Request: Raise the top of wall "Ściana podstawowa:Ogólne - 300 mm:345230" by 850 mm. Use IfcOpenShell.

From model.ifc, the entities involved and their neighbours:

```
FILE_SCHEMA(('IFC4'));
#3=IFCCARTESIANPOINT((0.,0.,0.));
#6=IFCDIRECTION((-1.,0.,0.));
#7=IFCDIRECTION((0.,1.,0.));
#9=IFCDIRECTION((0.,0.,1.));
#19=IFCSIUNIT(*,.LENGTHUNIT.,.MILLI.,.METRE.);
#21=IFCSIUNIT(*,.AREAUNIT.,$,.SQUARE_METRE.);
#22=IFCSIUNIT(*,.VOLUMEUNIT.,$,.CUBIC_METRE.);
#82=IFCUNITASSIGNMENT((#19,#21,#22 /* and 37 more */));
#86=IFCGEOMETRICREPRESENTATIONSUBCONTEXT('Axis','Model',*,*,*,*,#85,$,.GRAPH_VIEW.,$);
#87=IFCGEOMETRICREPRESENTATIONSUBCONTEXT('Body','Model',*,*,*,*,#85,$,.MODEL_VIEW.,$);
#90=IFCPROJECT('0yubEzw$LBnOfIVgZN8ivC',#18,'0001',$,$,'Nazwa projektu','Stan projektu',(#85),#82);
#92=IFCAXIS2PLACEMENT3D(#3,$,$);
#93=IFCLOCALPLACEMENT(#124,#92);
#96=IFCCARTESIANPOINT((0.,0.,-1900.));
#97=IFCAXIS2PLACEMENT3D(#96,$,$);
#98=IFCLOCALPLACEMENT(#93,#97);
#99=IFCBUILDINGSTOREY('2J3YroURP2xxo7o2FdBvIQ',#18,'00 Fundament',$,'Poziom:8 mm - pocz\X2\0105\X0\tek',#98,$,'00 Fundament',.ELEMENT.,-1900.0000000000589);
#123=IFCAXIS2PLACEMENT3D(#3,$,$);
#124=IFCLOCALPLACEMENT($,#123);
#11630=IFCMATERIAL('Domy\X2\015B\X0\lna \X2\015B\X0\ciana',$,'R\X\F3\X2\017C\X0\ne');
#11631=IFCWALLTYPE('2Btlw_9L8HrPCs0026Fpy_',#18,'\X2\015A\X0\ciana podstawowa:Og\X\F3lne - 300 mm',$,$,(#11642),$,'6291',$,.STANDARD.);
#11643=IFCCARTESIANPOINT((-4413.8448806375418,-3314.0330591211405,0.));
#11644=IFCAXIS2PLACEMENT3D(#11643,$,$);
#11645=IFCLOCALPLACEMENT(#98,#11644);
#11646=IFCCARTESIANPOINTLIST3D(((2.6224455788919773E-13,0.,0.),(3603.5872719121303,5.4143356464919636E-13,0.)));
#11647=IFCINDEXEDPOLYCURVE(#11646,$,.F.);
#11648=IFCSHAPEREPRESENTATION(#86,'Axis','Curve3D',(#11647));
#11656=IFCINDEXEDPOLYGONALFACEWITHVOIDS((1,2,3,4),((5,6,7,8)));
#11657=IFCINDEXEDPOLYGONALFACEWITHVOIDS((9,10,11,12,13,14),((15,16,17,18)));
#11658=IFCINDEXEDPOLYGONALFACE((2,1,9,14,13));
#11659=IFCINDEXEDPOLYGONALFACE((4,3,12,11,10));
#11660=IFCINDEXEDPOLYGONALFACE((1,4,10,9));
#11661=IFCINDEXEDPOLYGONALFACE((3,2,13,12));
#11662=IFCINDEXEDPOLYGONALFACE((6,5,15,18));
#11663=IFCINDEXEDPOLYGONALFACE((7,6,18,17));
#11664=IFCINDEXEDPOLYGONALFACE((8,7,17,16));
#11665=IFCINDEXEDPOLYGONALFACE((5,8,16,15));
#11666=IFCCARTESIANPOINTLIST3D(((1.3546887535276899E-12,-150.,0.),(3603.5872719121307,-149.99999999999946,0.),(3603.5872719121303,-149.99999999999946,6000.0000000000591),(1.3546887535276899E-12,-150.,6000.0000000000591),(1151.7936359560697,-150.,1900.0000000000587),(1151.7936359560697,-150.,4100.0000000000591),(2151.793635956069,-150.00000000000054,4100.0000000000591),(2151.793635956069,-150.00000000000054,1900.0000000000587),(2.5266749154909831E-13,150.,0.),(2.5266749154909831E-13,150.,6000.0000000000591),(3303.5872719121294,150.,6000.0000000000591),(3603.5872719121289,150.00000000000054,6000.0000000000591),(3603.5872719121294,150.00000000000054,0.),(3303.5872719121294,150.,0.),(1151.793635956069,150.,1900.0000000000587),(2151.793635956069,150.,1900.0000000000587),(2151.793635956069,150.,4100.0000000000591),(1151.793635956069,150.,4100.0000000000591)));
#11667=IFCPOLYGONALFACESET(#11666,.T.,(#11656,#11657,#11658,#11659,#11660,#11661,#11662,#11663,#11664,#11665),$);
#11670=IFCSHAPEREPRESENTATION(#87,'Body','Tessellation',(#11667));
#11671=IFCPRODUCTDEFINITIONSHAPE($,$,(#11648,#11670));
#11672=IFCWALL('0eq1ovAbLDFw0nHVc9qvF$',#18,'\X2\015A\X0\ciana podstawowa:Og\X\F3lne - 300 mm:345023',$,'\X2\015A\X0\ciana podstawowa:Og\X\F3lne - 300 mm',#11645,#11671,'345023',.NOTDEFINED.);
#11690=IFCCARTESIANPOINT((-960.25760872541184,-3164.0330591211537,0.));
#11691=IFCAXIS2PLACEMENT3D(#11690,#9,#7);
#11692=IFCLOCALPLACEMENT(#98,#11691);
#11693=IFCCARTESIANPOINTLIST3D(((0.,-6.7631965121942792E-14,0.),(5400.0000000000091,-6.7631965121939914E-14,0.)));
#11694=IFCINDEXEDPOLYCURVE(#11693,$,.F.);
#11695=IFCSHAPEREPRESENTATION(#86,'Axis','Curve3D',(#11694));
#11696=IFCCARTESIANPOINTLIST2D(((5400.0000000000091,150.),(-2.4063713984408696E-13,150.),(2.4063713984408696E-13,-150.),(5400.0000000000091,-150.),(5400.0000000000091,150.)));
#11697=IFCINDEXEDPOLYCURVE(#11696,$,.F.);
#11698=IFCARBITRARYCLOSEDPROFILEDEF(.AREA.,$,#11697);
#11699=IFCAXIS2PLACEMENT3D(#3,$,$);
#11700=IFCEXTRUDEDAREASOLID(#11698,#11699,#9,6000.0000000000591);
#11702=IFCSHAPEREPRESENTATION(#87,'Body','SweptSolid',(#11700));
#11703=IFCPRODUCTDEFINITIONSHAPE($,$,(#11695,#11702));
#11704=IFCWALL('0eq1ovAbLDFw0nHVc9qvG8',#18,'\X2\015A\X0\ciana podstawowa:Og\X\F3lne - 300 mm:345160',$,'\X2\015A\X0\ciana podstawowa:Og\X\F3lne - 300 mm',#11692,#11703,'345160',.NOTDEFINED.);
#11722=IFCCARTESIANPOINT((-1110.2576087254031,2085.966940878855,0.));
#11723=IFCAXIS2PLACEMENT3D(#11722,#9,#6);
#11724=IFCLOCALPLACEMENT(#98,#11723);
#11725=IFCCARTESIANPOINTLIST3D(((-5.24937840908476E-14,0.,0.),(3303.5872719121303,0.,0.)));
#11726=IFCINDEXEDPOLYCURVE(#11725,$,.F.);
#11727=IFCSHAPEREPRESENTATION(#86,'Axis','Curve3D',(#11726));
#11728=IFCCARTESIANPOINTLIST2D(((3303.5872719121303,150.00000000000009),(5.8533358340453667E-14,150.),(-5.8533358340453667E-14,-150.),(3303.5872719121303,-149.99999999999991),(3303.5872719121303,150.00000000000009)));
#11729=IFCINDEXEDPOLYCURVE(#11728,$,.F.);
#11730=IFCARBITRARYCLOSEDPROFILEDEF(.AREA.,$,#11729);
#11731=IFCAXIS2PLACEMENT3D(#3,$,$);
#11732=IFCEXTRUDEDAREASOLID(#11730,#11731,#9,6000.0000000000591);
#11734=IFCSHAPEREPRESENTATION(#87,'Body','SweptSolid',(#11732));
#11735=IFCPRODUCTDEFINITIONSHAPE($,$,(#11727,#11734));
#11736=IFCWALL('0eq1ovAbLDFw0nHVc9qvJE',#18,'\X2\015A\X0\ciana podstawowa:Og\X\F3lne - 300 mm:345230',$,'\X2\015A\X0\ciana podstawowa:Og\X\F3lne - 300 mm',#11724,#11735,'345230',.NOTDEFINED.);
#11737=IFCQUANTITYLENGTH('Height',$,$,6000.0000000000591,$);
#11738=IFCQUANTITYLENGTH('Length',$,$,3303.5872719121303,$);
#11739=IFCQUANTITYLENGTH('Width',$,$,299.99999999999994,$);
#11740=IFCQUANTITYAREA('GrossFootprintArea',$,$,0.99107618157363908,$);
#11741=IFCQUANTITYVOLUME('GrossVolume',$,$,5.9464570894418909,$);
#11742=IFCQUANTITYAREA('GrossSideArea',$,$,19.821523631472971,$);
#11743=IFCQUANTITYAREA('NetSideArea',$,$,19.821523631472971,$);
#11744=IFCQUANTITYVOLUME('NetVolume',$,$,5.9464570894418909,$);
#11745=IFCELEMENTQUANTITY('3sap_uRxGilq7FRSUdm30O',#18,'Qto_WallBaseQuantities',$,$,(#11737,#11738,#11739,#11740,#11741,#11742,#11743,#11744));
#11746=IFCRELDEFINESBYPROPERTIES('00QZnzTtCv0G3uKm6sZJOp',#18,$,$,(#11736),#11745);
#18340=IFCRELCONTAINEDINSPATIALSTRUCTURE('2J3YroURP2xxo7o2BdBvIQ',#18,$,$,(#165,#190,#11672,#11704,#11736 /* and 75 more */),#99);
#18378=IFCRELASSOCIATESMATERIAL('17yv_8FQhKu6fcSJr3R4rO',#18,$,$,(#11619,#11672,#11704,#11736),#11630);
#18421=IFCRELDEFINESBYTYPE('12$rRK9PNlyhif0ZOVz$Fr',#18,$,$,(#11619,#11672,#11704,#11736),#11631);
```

```python
import ifcopenshell
import ifcopenshell.api.pset
import ifcopenshell.geom
import ifcopenshell.util.element
import ifcopenshell.util.representation
import ifcopenshell.util.shape
import ifcopenshell.util.unit

model = ifcopenshell.open("model.ifc")
unit_scale = ifcopenshell.util.unit.calculate_unit_scale(model)
area_scale = ifcopenshell.util.unit.calculate_unit_scale(model, "AREAUNIT")
volume_scale = ifcopenshell.util.unit.calculate_unit_scale(model, "VOLUMEUNIT")
settings = ifcopenshell.geom.settings()


def volume(element):
    """Net volume in cubic metres, openings subtracted."""
    shape = ifcopenshell.geom.create_shape(settings, element)
    return ifcopenshell.util.shape.get_volume(shape.geometry)


wall = model.by_id(11736)
before = volume(wall)

body = ifcopenshell.util.representation.get_representation(wall, "Model", "Body")
solid = body.Items[0]
old_height = solid.Depth
solid.Depth += 0.85 / unit_scale
after = volume(wall)
thickness = 0.3  # wall thickness in metres

# Update the stored height, areas and volumes.
qto = model.by_id(ifcopenshell.util.element.get_pset(wall, "Qto_WallBaseQuantities", should_inherit=False)["id"])
ifcopenshell.api.pset.edit_qto(model, qto=qto, properties={
    "Height": solid.Depth,
    "GrossVolume": ifcopenshell.util.element.get_pset(wall, "Qto_WallBaseQuantities", "GrossVolume") * solid.Depth / old_height,
    "GrossSideArea": ifcopenshell.util.element.get_pset(wall, "Qto_WallBaseQuantities", "GrossSideArea") * solid.Depth / old_height,
    "NetSideArea": after / thickness / area_scale,
    "NetVolume": after / volume_scale,
})

print(f"height {old_height:g} -> {solid.Depth:g}, volume {before:.3f} -> {after:.3f} m3")

model.write("model_updated.ifc")
```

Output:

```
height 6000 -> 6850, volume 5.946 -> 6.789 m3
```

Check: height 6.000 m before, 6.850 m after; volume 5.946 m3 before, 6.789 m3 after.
